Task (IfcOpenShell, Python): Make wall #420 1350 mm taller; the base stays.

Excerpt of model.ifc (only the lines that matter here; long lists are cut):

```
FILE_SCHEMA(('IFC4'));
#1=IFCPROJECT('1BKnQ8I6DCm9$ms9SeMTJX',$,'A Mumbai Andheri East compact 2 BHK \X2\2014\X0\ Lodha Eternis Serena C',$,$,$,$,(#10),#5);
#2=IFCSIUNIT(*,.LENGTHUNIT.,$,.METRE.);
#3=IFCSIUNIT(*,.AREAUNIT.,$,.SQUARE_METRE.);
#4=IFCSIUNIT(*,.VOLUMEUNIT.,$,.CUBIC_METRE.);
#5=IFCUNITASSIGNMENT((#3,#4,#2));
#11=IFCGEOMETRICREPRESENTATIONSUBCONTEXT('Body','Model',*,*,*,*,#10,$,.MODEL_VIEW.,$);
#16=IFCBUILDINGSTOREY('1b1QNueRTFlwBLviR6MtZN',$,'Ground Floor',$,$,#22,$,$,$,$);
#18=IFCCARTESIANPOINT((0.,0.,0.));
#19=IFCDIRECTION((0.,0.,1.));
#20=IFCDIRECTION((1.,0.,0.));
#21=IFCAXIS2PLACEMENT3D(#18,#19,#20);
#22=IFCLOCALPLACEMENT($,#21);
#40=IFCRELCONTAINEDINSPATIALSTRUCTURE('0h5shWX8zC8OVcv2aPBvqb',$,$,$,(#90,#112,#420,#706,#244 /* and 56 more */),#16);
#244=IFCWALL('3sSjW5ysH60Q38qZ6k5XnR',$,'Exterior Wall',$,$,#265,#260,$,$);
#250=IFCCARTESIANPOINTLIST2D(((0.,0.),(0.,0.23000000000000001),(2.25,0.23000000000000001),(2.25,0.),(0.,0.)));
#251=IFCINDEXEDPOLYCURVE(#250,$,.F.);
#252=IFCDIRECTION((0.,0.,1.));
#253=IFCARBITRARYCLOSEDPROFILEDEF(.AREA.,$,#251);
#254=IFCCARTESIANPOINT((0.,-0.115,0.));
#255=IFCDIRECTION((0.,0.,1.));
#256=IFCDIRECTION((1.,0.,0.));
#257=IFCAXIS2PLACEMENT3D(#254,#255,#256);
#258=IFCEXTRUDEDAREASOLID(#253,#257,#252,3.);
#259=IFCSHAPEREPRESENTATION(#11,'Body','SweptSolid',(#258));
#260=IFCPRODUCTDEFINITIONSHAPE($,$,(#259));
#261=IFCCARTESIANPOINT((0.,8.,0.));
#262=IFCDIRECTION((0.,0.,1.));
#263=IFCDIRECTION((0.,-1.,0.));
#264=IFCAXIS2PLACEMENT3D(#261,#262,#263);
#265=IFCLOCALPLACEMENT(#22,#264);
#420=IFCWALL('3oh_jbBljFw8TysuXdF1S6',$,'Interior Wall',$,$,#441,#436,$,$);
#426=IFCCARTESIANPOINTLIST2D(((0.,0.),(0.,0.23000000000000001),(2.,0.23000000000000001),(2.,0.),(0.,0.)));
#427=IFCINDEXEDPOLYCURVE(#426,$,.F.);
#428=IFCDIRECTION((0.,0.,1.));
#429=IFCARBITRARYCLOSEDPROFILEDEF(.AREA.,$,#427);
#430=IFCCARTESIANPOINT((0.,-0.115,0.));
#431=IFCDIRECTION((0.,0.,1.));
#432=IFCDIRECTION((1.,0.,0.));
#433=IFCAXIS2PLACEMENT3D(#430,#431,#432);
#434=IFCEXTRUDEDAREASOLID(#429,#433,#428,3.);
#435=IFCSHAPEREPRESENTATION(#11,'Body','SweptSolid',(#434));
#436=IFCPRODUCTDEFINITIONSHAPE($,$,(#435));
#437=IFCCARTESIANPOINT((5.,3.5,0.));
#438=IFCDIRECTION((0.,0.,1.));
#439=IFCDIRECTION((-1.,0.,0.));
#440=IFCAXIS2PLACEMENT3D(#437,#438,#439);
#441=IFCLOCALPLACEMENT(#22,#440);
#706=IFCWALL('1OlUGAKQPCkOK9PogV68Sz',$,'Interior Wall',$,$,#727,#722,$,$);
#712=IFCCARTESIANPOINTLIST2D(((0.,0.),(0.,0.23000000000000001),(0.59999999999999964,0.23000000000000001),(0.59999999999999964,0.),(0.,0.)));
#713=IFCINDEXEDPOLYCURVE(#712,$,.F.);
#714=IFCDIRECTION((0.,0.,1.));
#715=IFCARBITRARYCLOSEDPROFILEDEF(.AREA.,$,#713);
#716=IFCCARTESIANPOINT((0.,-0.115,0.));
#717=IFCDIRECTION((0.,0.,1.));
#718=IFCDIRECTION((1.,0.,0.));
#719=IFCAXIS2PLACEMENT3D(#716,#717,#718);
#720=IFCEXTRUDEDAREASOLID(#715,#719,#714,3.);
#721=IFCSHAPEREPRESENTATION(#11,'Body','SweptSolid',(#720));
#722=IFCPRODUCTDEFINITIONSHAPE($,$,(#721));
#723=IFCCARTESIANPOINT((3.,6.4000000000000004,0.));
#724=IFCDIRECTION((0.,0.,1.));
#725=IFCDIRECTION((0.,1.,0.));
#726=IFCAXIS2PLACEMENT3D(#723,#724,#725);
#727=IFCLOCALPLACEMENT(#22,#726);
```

```python
import ifcopenshell
import ifcopenshell.geom
import ifcopenshell.util.representation
import ifcopenshell.util.shape

model = ifcopenshell.open("model.ifc")
settings = ifcopenshell.geom.settings()


def volume(element):
    """Net volume in cubic metres, openings subtracted."""
    shape = ifcopenshell.geom.create_shape(settings, element)
    return ifcopenshell.util.shape.get_volume(shape.geometry)


wall = model.by_guid("3oh_jbBljFw8TysuXdF1S6")
before = volume(wall)

body = ifcopenshell.util.representation.get_representation(wall, "Model", "Body")
solid = body.Items[0]
old_height = solid.Depth
solid.Depth += 1.35
after = volume(wall)

print(f"height {old_height:g} -> {solid.Depth:g}, volume {before:.3f} -> {after:.3f} m3")

model.write("model_v2.ifc")
```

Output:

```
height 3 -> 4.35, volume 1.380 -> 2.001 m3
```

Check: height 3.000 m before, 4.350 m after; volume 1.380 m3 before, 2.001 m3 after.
